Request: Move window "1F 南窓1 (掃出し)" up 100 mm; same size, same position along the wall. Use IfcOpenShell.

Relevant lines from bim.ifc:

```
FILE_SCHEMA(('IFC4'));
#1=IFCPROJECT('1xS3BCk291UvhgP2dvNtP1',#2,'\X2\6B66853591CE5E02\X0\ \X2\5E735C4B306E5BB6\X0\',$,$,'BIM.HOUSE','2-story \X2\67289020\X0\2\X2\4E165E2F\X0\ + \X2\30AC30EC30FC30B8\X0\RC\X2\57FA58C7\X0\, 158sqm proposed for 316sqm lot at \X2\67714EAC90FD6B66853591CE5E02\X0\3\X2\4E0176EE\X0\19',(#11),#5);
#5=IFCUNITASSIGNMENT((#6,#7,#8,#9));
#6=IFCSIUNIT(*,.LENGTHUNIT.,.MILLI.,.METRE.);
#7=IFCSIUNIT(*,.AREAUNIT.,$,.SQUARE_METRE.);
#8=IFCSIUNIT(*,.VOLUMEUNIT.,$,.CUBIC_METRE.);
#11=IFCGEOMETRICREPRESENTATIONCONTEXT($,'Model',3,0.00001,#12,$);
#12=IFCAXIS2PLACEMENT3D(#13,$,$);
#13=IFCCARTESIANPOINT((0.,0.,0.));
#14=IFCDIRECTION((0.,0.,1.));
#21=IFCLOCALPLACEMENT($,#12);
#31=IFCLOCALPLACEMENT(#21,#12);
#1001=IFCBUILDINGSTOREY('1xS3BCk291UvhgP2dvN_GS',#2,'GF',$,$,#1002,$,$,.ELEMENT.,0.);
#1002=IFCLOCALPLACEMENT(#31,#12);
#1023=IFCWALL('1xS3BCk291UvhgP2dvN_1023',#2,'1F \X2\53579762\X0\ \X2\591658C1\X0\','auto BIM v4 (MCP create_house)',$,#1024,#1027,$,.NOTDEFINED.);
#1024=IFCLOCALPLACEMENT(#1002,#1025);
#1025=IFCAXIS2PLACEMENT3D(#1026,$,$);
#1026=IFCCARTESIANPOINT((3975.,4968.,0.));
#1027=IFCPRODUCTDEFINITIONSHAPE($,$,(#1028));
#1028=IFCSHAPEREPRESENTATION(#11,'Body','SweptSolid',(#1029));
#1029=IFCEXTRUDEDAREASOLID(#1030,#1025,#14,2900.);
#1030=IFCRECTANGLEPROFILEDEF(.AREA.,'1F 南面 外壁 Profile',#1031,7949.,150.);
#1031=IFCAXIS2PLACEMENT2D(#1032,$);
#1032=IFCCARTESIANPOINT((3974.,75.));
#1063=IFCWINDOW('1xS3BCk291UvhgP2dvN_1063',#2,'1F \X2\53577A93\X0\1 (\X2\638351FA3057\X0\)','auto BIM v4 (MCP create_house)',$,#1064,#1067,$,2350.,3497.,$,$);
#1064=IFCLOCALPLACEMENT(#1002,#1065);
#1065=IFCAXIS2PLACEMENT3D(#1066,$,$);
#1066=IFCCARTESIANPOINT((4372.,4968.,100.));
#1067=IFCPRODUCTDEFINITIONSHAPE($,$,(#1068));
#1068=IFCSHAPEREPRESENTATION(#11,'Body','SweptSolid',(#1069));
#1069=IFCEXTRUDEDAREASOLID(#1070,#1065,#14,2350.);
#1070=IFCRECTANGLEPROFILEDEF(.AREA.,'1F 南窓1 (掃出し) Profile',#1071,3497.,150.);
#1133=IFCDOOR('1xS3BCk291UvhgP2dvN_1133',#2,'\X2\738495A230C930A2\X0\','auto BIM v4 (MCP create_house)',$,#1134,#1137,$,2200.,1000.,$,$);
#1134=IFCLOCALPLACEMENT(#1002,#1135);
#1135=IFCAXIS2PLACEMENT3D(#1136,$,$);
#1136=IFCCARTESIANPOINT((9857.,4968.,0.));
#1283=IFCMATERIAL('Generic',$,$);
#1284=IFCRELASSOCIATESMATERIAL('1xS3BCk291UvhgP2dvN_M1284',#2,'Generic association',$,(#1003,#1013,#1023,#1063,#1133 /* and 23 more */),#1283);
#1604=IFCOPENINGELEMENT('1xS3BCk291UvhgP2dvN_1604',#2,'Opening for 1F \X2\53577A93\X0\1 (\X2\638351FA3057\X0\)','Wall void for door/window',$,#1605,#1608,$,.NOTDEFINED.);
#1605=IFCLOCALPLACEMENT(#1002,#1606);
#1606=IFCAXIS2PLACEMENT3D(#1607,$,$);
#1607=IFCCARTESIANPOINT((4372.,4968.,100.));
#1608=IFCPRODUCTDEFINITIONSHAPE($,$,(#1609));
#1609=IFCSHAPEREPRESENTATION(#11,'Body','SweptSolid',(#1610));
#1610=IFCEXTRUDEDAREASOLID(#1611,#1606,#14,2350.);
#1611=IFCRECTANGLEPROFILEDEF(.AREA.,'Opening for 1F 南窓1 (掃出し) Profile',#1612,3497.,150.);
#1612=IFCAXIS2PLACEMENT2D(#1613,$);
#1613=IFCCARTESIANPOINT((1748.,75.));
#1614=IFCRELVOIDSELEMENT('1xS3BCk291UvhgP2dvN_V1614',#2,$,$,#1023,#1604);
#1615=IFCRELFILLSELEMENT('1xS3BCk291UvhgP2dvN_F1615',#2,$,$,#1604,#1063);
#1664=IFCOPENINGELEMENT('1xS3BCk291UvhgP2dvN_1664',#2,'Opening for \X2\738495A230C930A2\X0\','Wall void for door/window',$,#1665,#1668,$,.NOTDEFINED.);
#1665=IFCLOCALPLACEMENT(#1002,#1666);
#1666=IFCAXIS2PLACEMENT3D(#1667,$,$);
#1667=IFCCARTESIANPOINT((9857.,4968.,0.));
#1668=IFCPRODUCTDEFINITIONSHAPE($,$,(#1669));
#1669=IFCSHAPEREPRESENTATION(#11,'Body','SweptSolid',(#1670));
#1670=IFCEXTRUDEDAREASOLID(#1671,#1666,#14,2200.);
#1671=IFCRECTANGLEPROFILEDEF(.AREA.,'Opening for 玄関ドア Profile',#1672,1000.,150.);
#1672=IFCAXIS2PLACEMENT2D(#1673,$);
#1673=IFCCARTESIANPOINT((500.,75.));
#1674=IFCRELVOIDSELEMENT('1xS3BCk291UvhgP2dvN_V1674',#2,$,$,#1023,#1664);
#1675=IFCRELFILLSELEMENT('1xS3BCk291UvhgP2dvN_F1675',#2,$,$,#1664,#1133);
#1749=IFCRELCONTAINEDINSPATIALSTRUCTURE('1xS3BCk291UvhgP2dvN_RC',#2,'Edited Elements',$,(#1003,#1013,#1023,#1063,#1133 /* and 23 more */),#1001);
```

```python
import numpy as np
import ifcopenshell
import ifcopenshell.api.geometry
import ifcopenshell.util.placement
import ifcopenshell.util.unit

model = ifcopenshell.open("bim.ifc")
unit_scale = ifcopenshell.util.unit.calculate_unit_scale(model)

window = model.by_guid("1xS3BCk291UvhgP2dvN_1063")
opening = window.FillsVoids[0].RelatingOpeningElement
dz = 100.0

shift = np.array([0.0, 0.0, dz])
# The window is not placed relative to its opening, so move both.
for product in (opening, window):
    matrix = ifcopenshell.util.placement.get_local_placement(product.ObjectPlacement)
    matrix[:3, 3] += shift
    ifcopenshell.api.geometry.edit_object_placement(model, product=product, matrix=matrix, is_si=False)

print(f"moved by {dz * unit_scale:+.3f} m")

model.write("bim_updated.ifc")
```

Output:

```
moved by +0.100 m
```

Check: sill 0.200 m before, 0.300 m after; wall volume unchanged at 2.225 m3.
